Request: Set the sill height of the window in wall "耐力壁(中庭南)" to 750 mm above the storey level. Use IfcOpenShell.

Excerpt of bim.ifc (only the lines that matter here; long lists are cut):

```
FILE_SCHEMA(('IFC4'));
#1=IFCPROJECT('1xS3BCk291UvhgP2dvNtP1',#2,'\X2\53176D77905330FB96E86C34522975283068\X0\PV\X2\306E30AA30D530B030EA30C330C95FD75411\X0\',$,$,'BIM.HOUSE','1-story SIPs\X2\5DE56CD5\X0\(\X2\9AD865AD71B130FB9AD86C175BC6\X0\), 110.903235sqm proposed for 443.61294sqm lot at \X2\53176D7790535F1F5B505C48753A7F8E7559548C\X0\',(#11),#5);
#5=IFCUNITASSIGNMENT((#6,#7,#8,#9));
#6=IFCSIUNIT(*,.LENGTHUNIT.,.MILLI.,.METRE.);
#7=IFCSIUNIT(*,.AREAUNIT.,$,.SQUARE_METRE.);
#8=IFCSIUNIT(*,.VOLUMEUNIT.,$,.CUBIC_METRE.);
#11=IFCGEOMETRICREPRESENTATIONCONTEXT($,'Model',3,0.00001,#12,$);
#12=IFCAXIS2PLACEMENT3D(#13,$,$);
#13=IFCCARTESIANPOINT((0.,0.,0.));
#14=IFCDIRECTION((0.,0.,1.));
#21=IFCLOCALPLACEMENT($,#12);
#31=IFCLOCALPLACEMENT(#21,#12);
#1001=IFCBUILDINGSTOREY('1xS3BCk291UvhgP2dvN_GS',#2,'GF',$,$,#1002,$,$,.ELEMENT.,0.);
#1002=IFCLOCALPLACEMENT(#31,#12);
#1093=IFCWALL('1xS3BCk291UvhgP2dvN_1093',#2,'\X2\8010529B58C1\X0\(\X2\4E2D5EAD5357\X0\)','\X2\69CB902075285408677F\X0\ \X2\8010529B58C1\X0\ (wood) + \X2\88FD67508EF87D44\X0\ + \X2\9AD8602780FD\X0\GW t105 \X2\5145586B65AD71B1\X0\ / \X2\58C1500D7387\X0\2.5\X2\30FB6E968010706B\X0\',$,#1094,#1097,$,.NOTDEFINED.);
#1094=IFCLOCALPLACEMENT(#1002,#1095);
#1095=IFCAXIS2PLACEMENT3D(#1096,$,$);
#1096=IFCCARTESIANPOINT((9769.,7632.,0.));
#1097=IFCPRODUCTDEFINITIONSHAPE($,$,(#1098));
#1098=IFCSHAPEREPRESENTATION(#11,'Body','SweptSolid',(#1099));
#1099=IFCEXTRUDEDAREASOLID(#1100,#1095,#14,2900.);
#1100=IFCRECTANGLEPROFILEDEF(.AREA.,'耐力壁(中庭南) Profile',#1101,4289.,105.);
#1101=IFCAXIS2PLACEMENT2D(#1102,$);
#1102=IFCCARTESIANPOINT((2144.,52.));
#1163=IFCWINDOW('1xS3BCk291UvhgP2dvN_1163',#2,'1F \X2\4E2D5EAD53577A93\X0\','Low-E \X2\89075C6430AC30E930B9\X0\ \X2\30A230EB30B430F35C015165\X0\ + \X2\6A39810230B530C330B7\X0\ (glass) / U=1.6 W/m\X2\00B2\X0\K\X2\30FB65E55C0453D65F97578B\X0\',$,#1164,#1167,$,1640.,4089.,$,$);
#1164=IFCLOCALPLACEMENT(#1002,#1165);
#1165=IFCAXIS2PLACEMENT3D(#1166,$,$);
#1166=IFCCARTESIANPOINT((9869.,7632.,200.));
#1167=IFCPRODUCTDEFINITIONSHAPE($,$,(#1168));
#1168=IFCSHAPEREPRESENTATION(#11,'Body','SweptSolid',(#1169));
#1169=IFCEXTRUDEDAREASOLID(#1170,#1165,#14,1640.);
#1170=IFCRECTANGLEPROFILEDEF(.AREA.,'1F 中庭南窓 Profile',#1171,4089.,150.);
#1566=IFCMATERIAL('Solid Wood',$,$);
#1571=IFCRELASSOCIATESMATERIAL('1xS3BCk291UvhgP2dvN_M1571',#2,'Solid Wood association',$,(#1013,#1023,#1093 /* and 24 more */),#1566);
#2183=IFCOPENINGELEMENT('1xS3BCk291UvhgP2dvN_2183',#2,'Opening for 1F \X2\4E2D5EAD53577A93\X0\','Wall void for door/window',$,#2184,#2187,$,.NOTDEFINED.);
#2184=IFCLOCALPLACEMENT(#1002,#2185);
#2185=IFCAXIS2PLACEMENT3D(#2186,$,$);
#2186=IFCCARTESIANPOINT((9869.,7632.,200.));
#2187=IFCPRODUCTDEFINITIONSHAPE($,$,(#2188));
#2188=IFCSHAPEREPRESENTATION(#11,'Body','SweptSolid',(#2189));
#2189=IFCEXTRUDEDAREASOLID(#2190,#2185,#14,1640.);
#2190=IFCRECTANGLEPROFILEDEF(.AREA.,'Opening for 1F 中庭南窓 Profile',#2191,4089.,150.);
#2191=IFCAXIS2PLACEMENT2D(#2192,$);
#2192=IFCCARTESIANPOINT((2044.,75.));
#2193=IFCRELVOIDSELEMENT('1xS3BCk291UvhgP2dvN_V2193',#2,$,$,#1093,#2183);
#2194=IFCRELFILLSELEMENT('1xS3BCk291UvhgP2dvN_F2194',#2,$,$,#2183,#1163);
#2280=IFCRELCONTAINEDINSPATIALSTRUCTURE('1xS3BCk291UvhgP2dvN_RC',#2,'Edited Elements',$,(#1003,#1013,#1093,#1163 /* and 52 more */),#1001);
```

```python
import numpy as np
import ifcopenshell
import ifcopenshell.api.geometry
import ifcopenshell.geom
import ifcopenshell.util.element
import ifcopenshell.util.placement
import ifcopenshell.util.shape
import ifcopenshell.util.unit

model = ifcopenshell.open("bim.ifc")
unit_scale = ifcopenshell.util.unit.calculate_unit_scale(model)

window = model.by_id(1163)
opening = window.FillsVoids[0].RelatingOpeningElement
storey = ifcopenshell.util.element.get_container(window, ifc_class="IfcBuildingStorey")
level = ifcopenshell.util.placement.get_local_placement(storey.ObjectPlacement)[2, 3]

# The opening's origin need not be at the sill, so measure its lowest point.
shape = ifcopenshell.geom.create_shape(ifcopenshell.geom.settings(), opening)
bottom = ifcopenshell.util.shape.get_shape_bottom_elevation(shape, shape.geometry) / unit_scale
dz = level + 750.0 - bottom

shift = np.array([0.0, 0.0, dz])
# The window is not placed relative to its opening, so move both.
for product in (opening, window):
    matrix = ifcopenshell.util.placement.get_local_placement(product.ObjectPlacement)
    matrix[:3, 3] += shift
    ifcopenshell.api.geometry.edit_object_placement(model, product=product, matrix=matrix, is_si=False)

print(f"moved by {dz * unit_scale:+.3f} m")

model.write("bim_v2.ifc")
```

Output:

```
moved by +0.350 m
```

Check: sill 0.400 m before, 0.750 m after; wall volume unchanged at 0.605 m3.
